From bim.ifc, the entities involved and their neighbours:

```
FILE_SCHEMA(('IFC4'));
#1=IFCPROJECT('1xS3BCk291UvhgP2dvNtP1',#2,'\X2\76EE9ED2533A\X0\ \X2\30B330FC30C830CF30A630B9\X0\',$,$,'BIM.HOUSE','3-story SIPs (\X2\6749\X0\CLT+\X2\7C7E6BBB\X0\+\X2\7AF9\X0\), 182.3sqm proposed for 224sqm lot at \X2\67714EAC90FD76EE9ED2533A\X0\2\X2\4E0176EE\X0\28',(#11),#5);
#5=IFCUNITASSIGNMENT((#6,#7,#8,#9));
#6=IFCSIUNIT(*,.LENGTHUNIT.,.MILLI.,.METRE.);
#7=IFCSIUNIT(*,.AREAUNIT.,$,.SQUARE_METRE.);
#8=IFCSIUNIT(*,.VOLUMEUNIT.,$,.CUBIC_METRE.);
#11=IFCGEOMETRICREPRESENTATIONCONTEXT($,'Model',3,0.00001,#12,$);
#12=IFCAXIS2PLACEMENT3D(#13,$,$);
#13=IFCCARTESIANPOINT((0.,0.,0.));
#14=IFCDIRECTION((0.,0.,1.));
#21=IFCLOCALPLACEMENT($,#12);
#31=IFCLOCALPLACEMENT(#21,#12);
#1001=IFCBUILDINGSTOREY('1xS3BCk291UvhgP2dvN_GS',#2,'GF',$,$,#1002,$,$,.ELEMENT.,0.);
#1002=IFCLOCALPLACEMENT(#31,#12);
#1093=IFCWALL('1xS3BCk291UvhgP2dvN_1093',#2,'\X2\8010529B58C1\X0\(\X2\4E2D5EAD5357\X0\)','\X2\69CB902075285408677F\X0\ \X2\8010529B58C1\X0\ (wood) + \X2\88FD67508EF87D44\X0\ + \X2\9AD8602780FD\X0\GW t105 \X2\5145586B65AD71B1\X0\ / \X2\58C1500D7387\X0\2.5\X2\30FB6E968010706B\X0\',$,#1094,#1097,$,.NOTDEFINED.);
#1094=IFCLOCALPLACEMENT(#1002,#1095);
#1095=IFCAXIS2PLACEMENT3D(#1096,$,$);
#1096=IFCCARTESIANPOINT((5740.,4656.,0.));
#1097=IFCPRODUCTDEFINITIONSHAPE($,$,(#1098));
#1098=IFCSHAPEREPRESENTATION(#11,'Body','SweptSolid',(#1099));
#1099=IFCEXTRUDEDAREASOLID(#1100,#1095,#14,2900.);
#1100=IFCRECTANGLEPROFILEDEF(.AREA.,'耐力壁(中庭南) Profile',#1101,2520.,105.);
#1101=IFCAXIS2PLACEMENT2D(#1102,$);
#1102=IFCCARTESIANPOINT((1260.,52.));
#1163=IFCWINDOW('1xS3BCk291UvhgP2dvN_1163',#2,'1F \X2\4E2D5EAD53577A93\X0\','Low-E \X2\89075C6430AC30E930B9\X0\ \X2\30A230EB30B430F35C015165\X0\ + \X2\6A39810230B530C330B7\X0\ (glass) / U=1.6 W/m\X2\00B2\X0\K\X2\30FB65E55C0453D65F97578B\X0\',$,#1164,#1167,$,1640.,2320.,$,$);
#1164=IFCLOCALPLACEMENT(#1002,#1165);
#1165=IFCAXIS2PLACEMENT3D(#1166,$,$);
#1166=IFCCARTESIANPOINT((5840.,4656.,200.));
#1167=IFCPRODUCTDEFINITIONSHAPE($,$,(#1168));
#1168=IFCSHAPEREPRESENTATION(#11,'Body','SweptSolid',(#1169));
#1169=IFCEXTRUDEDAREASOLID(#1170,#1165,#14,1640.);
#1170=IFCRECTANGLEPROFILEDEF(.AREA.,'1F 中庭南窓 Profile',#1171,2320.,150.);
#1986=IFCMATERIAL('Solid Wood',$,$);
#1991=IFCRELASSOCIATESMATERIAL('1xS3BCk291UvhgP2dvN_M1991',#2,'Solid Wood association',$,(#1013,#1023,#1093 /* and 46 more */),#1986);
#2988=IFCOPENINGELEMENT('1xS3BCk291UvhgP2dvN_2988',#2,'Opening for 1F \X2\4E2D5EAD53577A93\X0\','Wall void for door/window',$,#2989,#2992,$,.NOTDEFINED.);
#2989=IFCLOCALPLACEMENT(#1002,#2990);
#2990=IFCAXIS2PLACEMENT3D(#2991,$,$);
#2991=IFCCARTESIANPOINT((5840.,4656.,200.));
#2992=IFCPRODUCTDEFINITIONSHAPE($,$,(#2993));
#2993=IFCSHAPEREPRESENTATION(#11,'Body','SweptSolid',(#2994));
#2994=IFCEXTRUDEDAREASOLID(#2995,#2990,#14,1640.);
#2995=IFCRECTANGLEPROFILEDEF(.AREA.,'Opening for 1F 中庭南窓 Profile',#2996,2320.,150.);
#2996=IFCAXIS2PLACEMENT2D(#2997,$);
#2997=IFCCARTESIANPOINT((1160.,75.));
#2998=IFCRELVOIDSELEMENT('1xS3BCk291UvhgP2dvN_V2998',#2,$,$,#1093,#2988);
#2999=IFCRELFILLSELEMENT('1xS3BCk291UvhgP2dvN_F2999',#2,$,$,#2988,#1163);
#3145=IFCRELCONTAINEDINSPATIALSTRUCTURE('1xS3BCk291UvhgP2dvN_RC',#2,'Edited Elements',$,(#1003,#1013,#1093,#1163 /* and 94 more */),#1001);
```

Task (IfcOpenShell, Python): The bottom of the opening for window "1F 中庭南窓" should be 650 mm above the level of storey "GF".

```python
import numpy as np
import ifcopenshell
import ifcopenshell.api.geometry
import ifcopenshell.geom
import ifcopenshell.util.element
import ifcopenshell.util.placement
import ifcopenshell.util.shape
import ifcopenshell.util.unit

model = ifcopenshell.open("bim.ifc")
unit_scale = ifcopenshell.util.unit.calculate_unit_scale(model)

window = model.by_guid("1xS3BCk291UvhgP2dvN_1163")
opening = window.FillsVoids[0].RelatingOpeningElement
storey = ifcopenshell.util.element.get_container(window, ifc_class="IfcBuildingStorey")
level = ifcopenshell.util.placement.get_local_placement(storey.ObjectPlacement)[2, 3]

# The opening's origin need not be at the sill, so measure its lowest point.
shape = ifcopenshell.geom.create_shape(ifcopenshell.geom.settings(), opening)
bottom = ifcopenshell.util.shape.get_shape_bottom_elevation(shape, shape.geometry) / unit_scale
dz = level + 0.65 / unit_scale - bottom

shift = np.array([0.0, 0.0, dz])
# The window is not placed relative to its opening, so move both.
for product in (opening, window):
    matrix = ifcopenshell.util.placement.get_local_placement(product.ObjectPlacement)
    matrix[:3, 3] += shift
    ifcopenshell.api.geometry.edit_object_placement(model, product=product, matrix=matrix, is_si=False)

print(f"moved by {dz * unit_scale:+.3f} m")

model.write("bim_rev.ifc")
```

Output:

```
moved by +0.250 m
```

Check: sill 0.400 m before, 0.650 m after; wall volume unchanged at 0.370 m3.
